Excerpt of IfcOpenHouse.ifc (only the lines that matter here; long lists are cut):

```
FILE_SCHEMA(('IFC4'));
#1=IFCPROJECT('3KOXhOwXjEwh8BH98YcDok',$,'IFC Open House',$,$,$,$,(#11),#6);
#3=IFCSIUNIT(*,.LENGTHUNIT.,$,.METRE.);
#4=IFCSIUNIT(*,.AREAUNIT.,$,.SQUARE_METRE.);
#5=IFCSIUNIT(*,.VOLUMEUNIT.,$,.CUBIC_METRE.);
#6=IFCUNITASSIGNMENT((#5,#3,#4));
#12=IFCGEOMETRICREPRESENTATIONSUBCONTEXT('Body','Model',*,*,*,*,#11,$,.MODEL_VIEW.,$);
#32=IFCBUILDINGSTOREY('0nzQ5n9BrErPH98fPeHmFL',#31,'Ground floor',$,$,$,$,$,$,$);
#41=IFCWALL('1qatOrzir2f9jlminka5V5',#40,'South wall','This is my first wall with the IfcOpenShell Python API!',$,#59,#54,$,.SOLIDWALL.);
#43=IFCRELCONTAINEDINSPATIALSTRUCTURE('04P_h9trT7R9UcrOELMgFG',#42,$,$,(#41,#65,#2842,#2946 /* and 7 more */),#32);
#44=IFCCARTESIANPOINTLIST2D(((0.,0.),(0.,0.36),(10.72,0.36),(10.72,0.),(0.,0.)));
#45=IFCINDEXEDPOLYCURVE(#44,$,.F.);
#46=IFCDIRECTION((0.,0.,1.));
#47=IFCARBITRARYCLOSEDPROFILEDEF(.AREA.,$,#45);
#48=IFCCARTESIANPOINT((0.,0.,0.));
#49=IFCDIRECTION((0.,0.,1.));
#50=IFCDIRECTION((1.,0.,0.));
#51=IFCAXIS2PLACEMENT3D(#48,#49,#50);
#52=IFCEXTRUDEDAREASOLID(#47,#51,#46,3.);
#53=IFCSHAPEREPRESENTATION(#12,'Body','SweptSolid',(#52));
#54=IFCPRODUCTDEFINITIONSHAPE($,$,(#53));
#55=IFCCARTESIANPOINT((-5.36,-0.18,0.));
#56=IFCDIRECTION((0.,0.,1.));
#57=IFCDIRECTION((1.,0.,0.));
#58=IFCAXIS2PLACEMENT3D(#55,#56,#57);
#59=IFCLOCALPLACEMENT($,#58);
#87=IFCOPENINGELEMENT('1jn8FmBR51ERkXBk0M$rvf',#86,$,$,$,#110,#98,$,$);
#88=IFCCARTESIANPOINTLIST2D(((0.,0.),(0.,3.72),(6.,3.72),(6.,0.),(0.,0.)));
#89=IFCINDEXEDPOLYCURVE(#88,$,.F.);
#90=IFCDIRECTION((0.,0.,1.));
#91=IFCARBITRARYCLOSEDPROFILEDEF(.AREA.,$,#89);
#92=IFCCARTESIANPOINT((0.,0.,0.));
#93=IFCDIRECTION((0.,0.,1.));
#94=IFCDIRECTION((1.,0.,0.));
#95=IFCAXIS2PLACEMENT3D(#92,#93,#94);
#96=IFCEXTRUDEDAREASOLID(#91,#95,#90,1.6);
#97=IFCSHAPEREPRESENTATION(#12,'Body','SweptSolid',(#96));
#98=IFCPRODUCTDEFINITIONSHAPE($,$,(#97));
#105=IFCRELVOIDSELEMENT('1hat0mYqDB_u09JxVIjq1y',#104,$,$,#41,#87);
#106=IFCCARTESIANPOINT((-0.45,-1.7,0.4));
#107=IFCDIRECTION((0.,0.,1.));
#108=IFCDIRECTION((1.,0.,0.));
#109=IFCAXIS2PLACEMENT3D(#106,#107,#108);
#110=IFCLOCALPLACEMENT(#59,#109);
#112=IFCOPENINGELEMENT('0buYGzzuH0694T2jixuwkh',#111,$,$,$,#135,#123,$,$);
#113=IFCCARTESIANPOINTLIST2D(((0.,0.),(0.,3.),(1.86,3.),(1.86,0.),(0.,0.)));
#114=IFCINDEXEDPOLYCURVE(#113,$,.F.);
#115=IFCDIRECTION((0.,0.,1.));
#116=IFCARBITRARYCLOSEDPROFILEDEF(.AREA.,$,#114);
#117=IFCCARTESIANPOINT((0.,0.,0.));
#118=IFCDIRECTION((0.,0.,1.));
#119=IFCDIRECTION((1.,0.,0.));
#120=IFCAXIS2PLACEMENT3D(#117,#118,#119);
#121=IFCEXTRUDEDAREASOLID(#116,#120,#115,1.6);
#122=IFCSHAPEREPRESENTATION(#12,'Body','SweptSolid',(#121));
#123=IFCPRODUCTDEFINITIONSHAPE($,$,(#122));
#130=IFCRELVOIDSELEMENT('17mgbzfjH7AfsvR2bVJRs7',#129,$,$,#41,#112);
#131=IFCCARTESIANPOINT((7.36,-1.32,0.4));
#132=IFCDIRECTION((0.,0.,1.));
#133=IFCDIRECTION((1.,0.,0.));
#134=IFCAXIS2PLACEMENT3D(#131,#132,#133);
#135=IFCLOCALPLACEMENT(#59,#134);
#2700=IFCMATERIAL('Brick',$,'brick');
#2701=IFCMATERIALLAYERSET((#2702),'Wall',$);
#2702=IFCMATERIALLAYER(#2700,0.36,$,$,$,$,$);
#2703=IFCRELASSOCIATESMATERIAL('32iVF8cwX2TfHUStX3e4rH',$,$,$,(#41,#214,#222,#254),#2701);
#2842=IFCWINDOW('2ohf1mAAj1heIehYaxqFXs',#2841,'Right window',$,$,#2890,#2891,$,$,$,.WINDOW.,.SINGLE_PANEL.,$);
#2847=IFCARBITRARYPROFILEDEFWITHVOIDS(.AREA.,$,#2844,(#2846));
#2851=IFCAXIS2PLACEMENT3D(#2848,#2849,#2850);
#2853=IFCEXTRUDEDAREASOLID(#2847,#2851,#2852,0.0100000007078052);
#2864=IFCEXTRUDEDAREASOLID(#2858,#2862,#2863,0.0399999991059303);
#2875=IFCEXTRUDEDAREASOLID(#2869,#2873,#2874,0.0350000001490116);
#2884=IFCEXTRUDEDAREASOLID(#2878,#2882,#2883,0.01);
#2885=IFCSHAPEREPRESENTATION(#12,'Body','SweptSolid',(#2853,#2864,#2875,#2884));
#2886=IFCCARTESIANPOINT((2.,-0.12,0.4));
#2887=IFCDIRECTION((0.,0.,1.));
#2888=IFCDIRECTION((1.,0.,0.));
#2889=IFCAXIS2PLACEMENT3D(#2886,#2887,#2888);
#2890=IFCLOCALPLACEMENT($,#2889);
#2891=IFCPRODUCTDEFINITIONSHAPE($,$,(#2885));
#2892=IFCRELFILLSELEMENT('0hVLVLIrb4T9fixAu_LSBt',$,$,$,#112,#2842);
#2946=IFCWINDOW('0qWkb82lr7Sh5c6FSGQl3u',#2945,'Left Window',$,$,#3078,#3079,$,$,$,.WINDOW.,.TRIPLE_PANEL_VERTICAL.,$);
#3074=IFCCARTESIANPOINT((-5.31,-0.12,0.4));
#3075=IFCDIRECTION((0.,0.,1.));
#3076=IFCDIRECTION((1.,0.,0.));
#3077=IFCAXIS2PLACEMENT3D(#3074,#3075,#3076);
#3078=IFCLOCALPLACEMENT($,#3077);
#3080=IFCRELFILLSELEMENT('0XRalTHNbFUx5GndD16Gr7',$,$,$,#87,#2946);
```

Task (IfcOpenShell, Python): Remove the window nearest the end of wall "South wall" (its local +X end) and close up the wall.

```python
import ifcopenshell
import ifcopenshell.api.feature
import ifcopenshell.api.root
import ifcopenshell.geom
import ifcopenshell.util.shape

model = ifcopenshell.open("IfcOpenHouse.ifc")
settings = ifcopenshell.geom.settings()


def volume(element):
    """Net volume in cubic metres, openings subtracted."""
    shape = ifcopenshell.geom.create_shape(settings, element)
    return ifcopenshell.util.shape.get_volume(shape.geometry)


window = model.by_guid("2ohf1mAAj1heIehYaxqFXs")
opening = window.FillsVoids[0].RelatingOpeningElement
wall = opening.VoidsElements[0].RelatingBuildingElement
before = volume(wall)

ifcopenshell.api.root.remove_product(model, product=window)
ifcopenshell.api.feature.remove_feature(model, feature=opening)

after = volume(wall)

print(f"wall volume {before:.3f} -> {after:.3f} m3")

model.write("IfcOpenHouse_v2.ifc")
```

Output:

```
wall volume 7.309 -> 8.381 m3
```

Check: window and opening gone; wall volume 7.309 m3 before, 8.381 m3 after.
